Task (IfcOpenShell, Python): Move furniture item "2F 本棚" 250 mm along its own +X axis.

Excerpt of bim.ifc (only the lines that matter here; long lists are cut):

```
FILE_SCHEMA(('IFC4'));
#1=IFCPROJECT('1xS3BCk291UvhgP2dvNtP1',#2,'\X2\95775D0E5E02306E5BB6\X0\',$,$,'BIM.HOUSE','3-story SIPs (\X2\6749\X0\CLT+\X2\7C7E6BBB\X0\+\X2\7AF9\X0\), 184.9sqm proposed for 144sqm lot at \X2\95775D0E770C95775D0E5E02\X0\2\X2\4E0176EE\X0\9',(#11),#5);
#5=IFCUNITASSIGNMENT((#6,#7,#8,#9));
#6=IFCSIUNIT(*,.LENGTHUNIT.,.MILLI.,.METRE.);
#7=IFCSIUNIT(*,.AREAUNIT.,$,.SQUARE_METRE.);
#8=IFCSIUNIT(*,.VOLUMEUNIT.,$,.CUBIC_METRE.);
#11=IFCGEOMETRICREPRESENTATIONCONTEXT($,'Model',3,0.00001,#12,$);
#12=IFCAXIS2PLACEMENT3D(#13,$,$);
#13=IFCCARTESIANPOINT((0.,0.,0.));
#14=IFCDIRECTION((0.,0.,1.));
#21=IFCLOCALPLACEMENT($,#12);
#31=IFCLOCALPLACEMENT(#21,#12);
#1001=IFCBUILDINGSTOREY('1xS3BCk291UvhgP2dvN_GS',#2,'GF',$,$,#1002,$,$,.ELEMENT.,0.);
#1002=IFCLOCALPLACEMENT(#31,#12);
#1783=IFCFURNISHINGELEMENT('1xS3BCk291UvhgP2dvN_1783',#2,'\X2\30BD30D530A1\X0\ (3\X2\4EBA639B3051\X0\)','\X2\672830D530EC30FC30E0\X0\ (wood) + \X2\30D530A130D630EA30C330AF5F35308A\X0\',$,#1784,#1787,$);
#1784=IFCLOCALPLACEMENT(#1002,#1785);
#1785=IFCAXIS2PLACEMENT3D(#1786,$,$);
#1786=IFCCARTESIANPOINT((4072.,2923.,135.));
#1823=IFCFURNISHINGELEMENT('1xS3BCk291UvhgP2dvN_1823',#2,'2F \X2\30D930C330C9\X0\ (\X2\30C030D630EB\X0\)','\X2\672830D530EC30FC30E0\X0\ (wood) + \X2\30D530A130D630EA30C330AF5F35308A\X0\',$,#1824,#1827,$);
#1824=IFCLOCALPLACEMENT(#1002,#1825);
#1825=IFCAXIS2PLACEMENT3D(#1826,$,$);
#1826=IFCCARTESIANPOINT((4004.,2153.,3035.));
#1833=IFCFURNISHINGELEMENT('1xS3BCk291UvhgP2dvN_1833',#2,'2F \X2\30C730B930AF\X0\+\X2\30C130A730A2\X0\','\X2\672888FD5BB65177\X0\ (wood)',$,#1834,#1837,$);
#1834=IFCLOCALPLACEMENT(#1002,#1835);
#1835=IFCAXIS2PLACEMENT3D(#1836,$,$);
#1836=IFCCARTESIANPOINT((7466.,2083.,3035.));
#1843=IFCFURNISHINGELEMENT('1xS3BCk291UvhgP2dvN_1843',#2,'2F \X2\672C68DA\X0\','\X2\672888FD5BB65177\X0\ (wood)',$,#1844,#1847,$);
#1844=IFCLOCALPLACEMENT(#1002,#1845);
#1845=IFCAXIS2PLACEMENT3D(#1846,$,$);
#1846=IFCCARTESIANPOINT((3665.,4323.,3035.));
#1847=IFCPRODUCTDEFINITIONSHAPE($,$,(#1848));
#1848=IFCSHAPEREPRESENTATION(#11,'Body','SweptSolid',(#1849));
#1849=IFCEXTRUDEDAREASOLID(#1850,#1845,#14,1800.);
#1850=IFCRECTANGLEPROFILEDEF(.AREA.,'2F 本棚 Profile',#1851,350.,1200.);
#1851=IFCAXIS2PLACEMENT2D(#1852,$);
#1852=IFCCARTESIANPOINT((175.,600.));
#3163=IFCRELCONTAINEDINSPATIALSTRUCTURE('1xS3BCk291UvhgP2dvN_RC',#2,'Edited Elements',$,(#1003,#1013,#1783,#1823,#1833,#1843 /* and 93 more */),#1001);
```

```python
import ifcopenshell
import ifcopenshell.api.geometry
import ifcopenshell.util.placement
import ifcopenshell.util.unit

model = ifcopenshell.open("bim.ifc")
unit_scale = ifcopenshell.util.unit.calculate_unit_scale(model)

item = model.by_guid("1xS3BCk291UvhgP2dvN_1843")
matrix = ifcopenshell.util.placement.get_local_placement(item.ObjectPlacement)
matrix[:3, 3] += matrix[:3, 0] * 0.25 / unit_scale
ifcopenshell.api.geometry.edit_object_placement(model, product=item, matrix=matrix, is_si=False)

print(ifcopenshell.util.placement.get_local_placement(item.ObjectPlacement).round(3) + 0.0)

model.write("bim_rev.ifc")
```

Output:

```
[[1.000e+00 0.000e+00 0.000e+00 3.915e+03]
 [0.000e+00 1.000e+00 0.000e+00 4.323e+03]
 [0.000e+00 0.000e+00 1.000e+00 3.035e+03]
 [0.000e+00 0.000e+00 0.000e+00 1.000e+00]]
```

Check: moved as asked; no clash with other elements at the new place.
